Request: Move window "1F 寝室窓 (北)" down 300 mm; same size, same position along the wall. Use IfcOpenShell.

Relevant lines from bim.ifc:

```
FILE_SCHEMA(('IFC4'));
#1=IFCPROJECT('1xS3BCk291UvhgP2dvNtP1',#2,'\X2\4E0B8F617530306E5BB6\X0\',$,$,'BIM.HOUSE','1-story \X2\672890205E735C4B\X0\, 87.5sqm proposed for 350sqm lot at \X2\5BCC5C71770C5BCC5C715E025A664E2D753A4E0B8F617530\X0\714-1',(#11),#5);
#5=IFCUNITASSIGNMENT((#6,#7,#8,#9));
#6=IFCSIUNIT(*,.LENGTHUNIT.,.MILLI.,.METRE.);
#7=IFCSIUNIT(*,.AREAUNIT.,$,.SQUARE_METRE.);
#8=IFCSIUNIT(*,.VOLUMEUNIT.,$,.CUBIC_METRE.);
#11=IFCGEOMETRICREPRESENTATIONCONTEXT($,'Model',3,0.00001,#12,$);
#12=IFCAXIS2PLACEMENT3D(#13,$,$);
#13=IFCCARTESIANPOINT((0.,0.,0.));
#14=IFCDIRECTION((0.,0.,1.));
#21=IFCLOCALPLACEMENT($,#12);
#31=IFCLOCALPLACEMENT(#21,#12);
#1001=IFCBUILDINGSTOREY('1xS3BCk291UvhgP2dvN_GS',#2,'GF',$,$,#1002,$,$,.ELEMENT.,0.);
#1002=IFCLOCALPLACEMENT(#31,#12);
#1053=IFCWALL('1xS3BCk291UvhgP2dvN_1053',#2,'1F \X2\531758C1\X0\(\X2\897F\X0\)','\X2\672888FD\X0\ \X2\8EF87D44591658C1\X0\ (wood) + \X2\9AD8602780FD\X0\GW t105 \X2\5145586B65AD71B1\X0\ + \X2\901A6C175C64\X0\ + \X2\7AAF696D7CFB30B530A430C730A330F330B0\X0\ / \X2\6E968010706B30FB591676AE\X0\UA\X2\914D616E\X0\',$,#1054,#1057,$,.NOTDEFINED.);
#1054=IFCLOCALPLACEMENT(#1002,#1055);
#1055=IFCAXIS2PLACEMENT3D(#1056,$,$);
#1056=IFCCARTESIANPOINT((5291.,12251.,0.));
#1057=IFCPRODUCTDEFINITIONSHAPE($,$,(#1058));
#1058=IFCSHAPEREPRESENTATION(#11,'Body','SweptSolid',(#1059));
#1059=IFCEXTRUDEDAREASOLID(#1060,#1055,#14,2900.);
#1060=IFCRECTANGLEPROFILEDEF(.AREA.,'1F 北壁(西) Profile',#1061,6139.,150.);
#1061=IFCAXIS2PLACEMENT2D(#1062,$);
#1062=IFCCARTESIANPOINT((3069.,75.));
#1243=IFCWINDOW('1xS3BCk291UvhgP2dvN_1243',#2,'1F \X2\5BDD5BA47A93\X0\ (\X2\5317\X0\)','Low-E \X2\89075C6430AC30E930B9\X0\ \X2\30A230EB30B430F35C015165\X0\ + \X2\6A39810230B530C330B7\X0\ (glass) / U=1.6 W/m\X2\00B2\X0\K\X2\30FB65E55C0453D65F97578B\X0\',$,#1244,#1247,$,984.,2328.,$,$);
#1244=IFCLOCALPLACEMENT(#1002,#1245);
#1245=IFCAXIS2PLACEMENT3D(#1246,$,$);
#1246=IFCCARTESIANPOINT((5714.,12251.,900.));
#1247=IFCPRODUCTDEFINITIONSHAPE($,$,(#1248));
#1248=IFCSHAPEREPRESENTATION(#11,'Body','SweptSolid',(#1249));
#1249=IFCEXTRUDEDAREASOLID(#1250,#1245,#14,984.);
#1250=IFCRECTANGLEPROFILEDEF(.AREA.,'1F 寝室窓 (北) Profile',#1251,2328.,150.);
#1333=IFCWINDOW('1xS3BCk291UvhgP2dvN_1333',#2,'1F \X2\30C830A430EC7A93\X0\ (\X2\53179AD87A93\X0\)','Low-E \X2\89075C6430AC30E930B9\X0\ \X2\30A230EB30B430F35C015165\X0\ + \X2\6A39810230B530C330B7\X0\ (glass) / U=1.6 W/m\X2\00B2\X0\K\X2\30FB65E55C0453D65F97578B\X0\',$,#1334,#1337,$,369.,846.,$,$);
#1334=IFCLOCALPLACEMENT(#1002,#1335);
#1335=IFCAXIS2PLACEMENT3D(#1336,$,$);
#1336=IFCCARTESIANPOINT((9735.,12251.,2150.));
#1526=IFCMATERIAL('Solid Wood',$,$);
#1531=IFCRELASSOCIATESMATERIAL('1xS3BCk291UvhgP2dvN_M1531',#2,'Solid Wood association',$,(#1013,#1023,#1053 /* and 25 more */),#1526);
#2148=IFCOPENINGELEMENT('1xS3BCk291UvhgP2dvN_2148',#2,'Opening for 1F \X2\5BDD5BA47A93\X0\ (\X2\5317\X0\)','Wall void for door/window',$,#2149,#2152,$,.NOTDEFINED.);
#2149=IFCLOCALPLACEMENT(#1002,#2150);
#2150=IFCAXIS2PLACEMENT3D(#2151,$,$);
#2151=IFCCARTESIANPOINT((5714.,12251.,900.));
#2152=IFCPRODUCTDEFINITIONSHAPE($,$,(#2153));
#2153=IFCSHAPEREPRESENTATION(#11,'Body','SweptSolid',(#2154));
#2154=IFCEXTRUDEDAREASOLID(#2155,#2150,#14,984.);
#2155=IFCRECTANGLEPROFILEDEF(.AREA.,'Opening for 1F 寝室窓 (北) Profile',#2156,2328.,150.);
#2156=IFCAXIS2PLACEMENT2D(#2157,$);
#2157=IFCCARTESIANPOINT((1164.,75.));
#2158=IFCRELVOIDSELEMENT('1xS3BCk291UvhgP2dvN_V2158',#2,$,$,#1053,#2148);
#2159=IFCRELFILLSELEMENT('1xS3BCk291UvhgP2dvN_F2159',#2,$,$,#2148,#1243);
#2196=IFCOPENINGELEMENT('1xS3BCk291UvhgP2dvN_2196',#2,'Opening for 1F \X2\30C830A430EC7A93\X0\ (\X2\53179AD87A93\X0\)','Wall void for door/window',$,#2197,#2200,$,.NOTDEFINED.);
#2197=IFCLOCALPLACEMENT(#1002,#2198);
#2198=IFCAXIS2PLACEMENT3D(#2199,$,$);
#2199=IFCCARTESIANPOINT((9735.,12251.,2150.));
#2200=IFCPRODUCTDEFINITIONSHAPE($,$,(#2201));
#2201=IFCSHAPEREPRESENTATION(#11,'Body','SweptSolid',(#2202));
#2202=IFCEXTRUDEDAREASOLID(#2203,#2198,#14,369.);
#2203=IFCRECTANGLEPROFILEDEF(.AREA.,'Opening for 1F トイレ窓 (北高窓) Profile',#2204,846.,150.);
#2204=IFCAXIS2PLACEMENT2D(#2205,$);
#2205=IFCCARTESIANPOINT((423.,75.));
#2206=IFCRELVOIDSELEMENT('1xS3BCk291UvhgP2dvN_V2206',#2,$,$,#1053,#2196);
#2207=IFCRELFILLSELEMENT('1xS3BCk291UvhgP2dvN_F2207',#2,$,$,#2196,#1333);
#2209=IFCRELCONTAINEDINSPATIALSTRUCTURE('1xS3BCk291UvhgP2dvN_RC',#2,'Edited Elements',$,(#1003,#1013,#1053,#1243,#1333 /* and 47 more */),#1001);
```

```python
import numpy as np
import ifcopenshell
import ifcopenshell.api.geometry
import ifcopenshell.util.placement
import ifcopenshell.util.unit

model = ifcopenshell.open("bim.ifc")
unit_scale = ifcopenshell.util.unit.calculate_unit_scale(model)

window = model.by_guid("1xS3BCk291UvhgP2dvN_1243")
opening = window.FillsVoids[0].RelatingOpeningElement
dz = -0.3 / unit_scale

shift = np.array([0.0, 0.0, dz])
# The window is not placed relative to its opening, so move both.
for product in (opening, window):
    matrix = ifcopenshell.util.placement.get_local_placement(product.ObjectPlacement)
    matrix[:3, 3] += shift
    ifcopenshell.api.geometry.edit_object_placement(model, product=product, matrix=matrix, is_si=False)

print(f"moved by {dz * unit_scale:+.3f} m")

model.write("bim-out.ifc")
```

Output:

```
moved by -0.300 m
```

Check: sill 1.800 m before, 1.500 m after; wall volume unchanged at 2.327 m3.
